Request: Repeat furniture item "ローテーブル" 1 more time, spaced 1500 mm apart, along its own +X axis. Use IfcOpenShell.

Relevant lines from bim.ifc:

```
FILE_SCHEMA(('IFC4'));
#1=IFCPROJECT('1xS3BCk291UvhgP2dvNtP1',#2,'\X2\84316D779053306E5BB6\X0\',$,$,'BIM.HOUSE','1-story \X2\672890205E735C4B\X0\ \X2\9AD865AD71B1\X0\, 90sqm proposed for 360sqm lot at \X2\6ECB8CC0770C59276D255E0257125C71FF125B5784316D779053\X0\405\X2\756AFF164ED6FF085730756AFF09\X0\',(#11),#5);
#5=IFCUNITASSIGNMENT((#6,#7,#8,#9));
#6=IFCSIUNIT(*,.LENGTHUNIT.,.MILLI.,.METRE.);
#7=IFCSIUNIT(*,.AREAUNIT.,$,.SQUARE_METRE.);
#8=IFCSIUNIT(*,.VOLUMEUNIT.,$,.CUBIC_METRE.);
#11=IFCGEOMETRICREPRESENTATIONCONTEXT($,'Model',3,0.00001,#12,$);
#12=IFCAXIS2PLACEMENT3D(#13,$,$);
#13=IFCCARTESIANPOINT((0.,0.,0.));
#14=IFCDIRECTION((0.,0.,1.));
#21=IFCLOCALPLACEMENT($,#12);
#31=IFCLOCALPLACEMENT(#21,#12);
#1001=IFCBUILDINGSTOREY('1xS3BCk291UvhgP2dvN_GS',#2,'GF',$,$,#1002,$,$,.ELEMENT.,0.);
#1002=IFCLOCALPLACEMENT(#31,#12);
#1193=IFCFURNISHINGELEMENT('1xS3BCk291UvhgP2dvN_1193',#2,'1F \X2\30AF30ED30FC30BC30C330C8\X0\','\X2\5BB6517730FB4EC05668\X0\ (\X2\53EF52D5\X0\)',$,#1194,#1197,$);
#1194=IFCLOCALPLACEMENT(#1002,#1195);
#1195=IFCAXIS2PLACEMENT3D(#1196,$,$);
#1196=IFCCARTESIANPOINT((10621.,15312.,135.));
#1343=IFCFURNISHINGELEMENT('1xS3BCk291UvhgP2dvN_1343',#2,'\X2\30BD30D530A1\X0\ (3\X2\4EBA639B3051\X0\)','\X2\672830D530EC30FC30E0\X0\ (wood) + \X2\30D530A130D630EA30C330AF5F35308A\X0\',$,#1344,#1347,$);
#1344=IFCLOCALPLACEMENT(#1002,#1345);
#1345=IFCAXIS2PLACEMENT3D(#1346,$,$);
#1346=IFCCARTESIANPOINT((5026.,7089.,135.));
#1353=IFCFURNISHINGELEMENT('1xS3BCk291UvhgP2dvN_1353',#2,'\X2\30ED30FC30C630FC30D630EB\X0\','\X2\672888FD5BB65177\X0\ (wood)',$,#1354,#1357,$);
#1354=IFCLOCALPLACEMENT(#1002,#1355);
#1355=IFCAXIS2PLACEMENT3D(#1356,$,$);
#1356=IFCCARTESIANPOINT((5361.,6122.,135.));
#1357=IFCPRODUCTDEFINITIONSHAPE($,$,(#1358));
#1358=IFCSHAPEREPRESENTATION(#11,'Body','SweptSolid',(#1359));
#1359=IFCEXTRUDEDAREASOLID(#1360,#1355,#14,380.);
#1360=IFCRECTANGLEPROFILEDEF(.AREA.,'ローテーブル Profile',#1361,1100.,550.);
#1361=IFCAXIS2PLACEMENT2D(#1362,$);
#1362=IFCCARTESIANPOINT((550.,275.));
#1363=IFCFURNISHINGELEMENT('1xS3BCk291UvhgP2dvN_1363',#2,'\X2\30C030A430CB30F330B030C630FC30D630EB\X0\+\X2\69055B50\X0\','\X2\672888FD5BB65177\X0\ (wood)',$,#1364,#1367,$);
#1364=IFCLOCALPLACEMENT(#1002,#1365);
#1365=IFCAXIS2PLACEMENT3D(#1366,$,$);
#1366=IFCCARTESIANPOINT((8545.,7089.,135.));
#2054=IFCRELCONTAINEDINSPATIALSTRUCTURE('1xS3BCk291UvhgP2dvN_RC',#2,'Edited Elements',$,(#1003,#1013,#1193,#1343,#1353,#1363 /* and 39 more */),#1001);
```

```python
import ifcopenshell
import ifcopenshell.api.geometry
import ifcopenshell.api.root
import ifcopenshell.util.element
import ifcopenshell.util.placement
import ifcopenshell.util.unit

model = ifcopenshell.open("bim.ifc")
unit_scale = ifcopenshell.util.unit.calculate_unit_scale(model)


def reuse_history(source, copy):
    """copy_class also copies each property set's owner history, people and application; keep the originals."""
    for rel in copy.IsDefinedBy:
        if rel.is_a("IfcRelDefinesByProperties") and (history := rel.RelatingPropertyDefinition.OwnerHistory):
            rel.RelatingPropertyDefinition.OwnerHistory = source.OwnerHistory
            ifcopenshell.util.element.remove_deep2(model, history)


source = model.by_id(1353)
base = ifcopenshell.util.placement.get_local_placement(source.ObjectPlacement)
step = base[:3, 0] * 1.5 / unit_scale

for i in range(1, 2):
    copy = ifcopenshell.api.root.copy_class(model, product=source)
    copy.Representation = ifcopenshell.util.element.copy_deep(
        model, source.Representation, exclude=["IfcGeometricRepresentationContext", "IfcRepresentationMap"]
    )
    reuse_history(source, copy)
    matrix = base.copy()
    matrix[:3, 3] += i * step
    print("added at", matrix[:3, 3].round(3) + 0.0)
    ifcopenshell.api.geometry.edit_object_placement(model, product=copy, matrix=matrix, is_si=False)

model.write("bim_rev.ifc")
```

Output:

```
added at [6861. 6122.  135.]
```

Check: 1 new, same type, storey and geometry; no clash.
